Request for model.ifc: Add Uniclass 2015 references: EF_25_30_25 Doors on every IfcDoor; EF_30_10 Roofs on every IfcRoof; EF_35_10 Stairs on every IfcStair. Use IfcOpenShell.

First a look at what the model holds.

```python
import ifcopenshell

model = ifcopenshell.open("model.ifc")
print(model.schema)
print("classifications:", [c.Name for c in model.by_type("IfcClassification")])
for ifc_class in ("IfcDoor", "IfcRoof", "IfcStair", "IfcWall", "IfcWindow"):
    print(ifc_class, len(model.by_type(ifc_class)))
```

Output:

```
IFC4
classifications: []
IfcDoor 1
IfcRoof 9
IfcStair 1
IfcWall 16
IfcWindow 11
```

```python
import ifcopenshell
import ifcopenshell.api.classification

model = ifcopenshell.open("model.ifc")

system = ifcopenshell.api.classification.add_classification(model, classification="Uniclass 2015")

codes = {
    "IfcDoor": ("EF_25_30_25", "Doors"),
    "IfcRoof": ("EF_30_10", "Roofs"),
    "IfcStair": ("EF_35_10", "Stairs"),
}
for ifc_class, (code, name) in codes.items():
    products = model.by_type(ifc_class)
    ifcopenshell.api.classification.add_reference(
        model, products=products, classification=system, identification=code, name=name
    )
    print(code, len(products))

model.write("model_edited.ifc")
```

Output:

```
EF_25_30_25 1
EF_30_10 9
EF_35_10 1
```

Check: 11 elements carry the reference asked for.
